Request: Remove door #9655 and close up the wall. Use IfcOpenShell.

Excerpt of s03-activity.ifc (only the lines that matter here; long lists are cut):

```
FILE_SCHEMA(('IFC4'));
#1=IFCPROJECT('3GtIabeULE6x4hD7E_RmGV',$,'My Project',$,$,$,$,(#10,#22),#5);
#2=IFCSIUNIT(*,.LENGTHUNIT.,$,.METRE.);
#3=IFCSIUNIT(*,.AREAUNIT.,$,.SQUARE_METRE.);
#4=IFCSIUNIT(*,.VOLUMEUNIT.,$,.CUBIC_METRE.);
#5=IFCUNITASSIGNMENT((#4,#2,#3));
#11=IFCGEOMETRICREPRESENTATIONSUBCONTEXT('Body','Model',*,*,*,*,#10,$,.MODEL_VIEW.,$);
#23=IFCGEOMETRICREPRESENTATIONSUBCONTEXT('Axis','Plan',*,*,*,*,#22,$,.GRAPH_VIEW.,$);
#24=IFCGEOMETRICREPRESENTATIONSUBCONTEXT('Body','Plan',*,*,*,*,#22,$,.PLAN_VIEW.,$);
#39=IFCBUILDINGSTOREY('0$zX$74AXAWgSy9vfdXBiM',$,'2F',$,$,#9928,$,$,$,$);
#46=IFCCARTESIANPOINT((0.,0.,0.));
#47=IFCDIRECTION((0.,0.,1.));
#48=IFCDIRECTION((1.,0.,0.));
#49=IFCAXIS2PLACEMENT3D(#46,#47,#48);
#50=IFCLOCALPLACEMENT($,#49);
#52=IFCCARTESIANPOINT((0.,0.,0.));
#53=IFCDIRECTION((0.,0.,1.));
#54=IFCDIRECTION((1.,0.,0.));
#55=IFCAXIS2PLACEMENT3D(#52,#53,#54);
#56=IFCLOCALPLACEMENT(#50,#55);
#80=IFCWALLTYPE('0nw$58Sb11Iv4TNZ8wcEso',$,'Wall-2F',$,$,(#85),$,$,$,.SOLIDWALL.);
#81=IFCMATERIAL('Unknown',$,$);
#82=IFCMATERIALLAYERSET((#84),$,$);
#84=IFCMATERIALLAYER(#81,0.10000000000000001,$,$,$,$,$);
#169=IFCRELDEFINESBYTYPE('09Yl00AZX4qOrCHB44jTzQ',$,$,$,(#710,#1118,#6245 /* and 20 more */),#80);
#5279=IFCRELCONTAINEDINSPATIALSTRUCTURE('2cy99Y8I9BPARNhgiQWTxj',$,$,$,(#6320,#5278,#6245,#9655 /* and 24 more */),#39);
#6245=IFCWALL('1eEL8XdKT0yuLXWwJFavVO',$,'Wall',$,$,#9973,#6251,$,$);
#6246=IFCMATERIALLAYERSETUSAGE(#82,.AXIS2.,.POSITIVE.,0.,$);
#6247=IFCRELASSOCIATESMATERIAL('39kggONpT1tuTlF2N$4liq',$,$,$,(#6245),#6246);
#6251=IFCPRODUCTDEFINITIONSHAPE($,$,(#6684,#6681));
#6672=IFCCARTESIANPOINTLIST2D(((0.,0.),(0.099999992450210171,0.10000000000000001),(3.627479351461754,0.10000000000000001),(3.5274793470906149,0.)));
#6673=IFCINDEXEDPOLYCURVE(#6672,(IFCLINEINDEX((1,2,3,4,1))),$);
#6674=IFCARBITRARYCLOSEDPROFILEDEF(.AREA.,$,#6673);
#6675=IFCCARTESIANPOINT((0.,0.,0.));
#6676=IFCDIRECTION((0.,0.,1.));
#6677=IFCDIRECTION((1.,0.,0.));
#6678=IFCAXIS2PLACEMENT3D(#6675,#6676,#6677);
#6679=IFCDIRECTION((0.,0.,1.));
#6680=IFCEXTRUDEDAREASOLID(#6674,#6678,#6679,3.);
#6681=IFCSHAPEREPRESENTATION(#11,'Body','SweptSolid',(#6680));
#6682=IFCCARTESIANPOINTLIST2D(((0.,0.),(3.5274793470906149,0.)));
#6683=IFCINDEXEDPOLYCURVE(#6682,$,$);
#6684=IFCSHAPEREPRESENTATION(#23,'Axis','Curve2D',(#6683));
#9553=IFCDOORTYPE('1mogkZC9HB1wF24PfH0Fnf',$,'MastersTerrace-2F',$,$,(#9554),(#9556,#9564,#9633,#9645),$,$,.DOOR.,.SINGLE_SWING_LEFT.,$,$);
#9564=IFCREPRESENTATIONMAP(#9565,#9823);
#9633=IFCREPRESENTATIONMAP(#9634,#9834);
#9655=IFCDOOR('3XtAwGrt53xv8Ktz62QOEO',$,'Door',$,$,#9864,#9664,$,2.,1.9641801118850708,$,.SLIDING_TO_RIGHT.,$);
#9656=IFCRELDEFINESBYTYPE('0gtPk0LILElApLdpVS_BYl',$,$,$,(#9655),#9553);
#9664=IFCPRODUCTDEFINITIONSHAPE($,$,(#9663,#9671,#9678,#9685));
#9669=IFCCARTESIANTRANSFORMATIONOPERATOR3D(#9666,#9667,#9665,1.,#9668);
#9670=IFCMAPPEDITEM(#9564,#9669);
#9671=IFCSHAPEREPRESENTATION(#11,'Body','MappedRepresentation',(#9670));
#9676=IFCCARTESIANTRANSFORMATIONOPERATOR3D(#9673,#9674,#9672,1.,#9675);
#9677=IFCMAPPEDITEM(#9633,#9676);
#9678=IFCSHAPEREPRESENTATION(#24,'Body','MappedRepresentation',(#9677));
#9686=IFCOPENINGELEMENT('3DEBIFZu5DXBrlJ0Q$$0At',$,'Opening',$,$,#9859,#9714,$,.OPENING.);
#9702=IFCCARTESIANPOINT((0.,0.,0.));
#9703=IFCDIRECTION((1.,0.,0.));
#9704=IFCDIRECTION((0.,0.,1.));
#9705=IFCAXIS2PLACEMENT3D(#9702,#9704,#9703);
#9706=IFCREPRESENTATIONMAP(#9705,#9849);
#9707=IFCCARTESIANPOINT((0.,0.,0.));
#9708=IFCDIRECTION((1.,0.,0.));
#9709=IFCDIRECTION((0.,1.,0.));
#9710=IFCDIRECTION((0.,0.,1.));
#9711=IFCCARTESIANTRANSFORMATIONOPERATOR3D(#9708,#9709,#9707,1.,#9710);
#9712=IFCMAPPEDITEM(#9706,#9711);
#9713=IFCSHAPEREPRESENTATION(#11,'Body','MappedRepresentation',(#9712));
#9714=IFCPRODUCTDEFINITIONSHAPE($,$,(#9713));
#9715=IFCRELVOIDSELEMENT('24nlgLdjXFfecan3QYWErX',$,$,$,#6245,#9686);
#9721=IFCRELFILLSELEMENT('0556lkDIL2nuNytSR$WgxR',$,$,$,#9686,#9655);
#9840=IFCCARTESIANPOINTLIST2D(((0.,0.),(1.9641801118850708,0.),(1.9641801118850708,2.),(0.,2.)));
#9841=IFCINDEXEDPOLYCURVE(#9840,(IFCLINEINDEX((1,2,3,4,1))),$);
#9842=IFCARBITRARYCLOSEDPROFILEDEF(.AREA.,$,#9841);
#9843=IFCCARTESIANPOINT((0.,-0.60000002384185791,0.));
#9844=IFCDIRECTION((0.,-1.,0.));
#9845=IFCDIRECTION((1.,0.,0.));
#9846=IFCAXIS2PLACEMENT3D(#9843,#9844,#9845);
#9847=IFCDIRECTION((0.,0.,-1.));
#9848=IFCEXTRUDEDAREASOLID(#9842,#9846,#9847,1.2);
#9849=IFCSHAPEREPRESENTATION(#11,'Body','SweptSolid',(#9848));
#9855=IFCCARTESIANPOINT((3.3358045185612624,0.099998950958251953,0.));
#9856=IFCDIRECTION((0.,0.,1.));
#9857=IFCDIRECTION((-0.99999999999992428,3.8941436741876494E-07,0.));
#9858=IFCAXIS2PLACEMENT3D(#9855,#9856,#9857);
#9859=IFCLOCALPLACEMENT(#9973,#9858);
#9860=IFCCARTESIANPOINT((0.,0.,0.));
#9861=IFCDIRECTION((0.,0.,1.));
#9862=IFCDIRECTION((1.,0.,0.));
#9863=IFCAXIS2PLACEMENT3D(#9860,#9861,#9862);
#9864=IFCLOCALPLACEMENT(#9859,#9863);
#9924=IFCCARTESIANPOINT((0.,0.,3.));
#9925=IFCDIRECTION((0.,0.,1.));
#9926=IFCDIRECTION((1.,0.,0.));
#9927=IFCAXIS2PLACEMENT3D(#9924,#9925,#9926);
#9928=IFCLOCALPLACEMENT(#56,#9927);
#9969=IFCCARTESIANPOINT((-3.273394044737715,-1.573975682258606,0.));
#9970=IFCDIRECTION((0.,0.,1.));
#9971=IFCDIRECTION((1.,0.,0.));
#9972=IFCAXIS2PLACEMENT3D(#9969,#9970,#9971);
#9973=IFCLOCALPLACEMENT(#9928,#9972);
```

```python
import ifcopenshell
import ifcopenshell.api.feature
import ifcopenshell.api.root
import ifcopenshell.geom
import ifcopenshell.util.shape

model = ifcopenshell.open("s03-activity.ifc")
settings = ifcopenshell.geom.settings()


def volume(element):
    """Net volume in cubic metres, openings subtracted."""
    shape = ifcopenshell.geom.create_shape(settings, element)
    return ifcopenshell.util.shape.get_volume(shape.geometry)


door = model.by_guid("3XtAwGrt53xv8Ktz62QOEO")
opening = door.FillsVoids[0].RelatingOpeningElement
wall = opening.VoidsElements[0].RelatingBuildingElement
before = volume(wall)

ifcopenshell.api.root.remove_product(model, product=door)
ifcopenshell.api.feature.remove_feature(model, feature=opening)

after = volume(wall)

print(f"wall volume {before:.3f} -> {after:.3f} m3")

model.write("s03-activity_updated.ifc")
```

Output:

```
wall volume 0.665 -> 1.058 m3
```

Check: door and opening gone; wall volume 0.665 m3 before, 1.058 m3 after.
